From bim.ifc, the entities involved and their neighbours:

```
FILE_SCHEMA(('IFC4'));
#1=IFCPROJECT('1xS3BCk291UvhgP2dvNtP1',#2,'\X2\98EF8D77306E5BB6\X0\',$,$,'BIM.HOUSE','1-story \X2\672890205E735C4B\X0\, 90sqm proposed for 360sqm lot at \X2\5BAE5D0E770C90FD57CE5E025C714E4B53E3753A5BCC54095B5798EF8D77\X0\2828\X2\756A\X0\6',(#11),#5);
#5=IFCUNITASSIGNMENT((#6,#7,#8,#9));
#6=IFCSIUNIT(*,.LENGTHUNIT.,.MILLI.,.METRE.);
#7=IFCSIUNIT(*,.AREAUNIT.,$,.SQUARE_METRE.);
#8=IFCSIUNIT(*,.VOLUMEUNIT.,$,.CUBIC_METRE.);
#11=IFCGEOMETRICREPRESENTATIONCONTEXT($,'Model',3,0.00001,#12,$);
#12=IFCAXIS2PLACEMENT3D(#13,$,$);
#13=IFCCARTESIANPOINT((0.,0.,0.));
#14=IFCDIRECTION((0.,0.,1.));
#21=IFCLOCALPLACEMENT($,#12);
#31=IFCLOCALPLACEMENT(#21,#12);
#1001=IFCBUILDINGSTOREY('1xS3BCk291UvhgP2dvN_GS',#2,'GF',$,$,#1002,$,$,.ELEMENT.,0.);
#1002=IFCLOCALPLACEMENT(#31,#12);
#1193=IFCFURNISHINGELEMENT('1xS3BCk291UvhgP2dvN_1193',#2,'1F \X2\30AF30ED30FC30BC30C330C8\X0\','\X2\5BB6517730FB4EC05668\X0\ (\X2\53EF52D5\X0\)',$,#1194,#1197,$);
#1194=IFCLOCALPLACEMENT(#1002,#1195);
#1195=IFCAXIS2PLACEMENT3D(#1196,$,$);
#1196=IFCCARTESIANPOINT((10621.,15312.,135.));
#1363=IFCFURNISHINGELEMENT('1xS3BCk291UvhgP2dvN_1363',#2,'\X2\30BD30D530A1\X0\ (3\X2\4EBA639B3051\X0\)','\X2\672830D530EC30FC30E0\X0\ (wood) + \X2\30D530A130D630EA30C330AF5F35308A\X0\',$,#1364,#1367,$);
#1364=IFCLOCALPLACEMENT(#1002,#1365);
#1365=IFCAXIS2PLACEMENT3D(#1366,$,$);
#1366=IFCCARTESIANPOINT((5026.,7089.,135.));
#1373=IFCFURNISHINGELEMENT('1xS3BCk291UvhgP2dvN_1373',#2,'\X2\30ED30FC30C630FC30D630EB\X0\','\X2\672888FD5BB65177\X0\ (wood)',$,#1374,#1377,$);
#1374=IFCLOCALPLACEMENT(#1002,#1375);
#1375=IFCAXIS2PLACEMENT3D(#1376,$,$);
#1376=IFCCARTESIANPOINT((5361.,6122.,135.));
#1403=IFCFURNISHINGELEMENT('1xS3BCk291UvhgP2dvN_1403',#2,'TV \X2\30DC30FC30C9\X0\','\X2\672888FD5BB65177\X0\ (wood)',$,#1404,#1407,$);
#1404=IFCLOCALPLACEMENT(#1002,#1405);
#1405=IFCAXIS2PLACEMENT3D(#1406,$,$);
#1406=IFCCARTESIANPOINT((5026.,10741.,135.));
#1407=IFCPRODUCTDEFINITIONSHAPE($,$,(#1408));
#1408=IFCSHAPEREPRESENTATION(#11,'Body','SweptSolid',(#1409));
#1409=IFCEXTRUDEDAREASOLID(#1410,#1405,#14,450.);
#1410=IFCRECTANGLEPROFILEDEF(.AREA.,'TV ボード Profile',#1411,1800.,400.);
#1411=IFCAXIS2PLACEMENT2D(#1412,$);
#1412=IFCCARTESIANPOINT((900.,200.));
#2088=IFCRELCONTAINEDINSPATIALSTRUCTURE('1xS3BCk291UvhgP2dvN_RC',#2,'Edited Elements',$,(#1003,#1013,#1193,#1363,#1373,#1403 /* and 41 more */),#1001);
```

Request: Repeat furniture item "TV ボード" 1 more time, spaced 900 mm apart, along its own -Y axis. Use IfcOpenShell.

```python
import ifcopenshell
import ifcopenshell.api.geometry
import ifcopenshell.api.root
import ifcopenshell.util.element
import ifcopenshell.util.placement
import ifcopenshell.util.unit

model = ifcopenshell.open("bim.ifc")
unit_scale = ifcopenshell.util.unit.calculate_unit_scale(model)


def reuse_history(source, copy):
    """copy_class also copies each property set's owner history, people and application; keep the originals."""
    for rel in copy.IsDefinedBy:
        if rel.is_a("IfcRelDefinesByProperties") and (history := rel.RelatingPropertyDefinition.OwnerHistory):
            rel.RelatingPropertyDefinition.OwnerHistory = source.OwnerHistory
            ifcopenshell.util.element.remove_deep2(model, history)


source = model.by_guid("1xS3BCk291UvhgP2dvN_1403")
base = ifcopenshell.util.placement.get_local_placement(source.ObjectPlacement)
step = -base[:3, 1] * 0.9 / unit_scale

for i in range(1, 2):
    copy = ifcopenshell.api.root.copy_class(model, product=source)
    copy.Representation = ifcopenshell.util.element.copy_deep(
        model, source.Representation, exclude=["IfcGeometricRepresentationContext", "IfcRepresentationMap"]
    )
    reuse_history(source, copy)
    matrix = base.copy()
    matrix[:3, 3] += i * step
    print("added at", matrix[:3, 3].round(3) + 0.0)
    ifcopenshell.api.geometry.edit_object_placement(model, product=copy, matrix=matrix, is_si=False)

model.write("bim_edited.ifc")
```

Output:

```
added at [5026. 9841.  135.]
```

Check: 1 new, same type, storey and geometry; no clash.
